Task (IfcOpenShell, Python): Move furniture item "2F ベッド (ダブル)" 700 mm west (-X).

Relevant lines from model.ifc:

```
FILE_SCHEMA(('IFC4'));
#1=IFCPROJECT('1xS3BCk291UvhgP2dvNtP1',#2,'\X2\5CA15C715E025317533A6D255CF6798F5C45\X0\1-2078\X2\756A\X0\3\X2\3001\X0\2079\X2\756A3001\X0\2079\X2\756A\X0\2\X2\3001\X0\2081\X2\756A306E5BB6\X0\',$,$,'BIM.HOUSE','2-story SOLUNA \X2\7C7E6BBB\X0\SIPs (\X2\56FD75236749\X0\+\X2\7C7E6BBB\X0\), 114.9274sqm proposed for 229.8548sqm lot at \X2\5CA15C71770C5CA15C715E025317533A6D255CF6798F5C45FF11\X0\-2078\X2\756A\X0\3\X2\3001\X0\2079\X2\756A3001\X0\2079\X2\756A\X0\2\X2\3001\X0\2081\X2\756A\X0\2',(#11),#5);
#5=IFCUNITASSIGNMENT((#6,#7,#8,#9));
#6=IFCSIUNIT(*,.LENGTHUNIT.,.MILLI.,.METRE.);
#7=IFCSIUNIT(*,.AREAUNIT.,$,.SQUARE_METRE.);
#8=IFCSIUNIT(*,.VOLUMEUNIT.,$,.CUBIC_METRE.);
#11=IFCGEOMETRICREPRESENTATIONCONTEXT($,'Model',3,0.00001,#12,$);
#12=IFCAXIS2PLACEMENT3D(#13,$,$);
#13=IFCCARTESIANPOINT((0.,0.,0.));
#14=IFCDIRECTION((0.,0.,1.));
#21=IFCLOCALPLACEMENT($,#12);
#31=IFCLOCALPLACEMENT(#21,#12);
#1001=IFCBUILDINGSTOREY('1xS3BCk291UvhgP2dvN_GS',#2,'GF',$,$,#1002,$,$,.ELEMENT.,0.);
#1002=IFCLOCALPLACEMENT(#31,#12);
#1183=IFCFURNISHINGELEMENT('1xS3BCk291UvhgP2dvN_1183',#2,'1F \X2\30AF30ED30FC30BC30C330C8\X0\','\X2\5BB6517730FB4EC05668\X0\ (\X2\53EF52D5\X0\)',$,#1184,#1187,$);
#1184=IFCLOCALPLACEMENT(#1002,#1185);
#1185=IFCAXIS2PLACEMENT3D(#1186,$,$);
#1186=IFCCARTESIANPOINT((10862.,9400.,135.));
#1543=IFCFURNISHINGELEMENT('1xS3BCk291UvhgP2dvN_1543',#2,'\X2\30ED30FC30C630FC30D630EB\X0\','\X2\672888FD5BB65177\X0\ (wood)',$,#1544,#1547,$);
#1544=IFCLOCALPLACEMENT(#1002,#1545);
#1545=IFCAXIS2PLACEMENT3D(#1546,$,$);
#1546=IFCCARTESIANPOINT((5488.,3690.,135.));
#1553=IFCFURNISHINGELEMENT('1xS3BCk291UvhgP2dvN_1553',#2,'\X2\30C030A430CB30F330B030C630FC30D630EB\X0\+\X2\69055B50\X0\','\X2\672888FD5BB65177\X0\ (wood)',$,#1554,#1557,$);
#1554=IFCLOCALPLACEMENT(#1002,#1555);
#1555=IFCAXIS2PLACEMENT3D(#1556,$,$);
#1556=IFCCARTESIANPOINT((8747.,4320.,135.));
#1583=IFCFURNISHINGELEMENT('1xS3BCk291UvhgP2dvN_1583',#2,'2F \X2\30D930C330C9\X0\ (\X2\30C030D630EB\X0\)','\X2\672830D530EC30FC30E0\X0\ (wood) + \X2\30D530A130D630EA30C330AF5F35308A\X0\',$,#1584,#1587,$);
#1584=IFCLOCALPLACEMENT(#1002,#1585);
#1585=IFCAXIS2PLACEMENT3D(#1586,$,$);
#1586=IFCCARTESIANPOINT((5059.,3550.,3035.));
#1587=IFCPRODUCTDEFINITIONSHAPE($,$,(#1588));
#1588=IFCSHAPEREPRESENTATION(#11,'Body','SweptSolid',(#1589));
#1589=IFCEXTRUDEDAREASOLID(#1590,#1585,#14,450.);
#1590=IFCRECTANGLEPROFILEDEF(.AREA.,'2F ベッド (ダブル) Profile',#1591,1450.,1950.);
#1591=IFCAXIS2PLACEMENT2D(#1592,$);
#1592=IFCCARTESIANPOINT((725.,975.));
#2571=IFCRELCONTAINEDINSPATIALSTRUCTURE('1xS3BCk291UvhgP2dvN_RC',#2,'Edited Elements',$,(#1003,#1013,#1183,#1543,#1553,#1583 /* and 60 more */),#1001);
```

```python
import ifcopenshell
import ifcopenshell.api.geometry
import ifcopenshell.util.placement
import ifcopenshell.util.unit

model = ifcopenshell.open("model.ifc")
unit_scale = ifcopenshell.util.unit.calculate_unit_scale(model)

item = model.by_guid("1xS3BCk291UvhgP2dvN_1583")
matrix = ifcopenshell.util.placement.get_local_placement(item.ObjectPlacement)
matrix[0, 3] -= 0.7 / unit_scale
ifcopenshell.api.geometry.edit_object_placement(model, product=item, matrix=matrix, is_si=False)

print(ifcopenshell.util.placement.get_local_placement(item.ObjectPlacement).round(3) + 0.0)

model.write("model_v2.ifc")
```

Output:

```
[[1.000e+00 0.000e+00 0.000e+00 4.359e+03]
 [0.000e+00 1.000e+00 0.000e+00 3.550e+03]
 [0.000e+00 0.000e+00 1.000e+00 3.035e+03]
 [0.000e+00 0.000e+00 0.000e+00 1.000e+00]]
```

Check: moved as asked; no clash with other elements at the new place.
